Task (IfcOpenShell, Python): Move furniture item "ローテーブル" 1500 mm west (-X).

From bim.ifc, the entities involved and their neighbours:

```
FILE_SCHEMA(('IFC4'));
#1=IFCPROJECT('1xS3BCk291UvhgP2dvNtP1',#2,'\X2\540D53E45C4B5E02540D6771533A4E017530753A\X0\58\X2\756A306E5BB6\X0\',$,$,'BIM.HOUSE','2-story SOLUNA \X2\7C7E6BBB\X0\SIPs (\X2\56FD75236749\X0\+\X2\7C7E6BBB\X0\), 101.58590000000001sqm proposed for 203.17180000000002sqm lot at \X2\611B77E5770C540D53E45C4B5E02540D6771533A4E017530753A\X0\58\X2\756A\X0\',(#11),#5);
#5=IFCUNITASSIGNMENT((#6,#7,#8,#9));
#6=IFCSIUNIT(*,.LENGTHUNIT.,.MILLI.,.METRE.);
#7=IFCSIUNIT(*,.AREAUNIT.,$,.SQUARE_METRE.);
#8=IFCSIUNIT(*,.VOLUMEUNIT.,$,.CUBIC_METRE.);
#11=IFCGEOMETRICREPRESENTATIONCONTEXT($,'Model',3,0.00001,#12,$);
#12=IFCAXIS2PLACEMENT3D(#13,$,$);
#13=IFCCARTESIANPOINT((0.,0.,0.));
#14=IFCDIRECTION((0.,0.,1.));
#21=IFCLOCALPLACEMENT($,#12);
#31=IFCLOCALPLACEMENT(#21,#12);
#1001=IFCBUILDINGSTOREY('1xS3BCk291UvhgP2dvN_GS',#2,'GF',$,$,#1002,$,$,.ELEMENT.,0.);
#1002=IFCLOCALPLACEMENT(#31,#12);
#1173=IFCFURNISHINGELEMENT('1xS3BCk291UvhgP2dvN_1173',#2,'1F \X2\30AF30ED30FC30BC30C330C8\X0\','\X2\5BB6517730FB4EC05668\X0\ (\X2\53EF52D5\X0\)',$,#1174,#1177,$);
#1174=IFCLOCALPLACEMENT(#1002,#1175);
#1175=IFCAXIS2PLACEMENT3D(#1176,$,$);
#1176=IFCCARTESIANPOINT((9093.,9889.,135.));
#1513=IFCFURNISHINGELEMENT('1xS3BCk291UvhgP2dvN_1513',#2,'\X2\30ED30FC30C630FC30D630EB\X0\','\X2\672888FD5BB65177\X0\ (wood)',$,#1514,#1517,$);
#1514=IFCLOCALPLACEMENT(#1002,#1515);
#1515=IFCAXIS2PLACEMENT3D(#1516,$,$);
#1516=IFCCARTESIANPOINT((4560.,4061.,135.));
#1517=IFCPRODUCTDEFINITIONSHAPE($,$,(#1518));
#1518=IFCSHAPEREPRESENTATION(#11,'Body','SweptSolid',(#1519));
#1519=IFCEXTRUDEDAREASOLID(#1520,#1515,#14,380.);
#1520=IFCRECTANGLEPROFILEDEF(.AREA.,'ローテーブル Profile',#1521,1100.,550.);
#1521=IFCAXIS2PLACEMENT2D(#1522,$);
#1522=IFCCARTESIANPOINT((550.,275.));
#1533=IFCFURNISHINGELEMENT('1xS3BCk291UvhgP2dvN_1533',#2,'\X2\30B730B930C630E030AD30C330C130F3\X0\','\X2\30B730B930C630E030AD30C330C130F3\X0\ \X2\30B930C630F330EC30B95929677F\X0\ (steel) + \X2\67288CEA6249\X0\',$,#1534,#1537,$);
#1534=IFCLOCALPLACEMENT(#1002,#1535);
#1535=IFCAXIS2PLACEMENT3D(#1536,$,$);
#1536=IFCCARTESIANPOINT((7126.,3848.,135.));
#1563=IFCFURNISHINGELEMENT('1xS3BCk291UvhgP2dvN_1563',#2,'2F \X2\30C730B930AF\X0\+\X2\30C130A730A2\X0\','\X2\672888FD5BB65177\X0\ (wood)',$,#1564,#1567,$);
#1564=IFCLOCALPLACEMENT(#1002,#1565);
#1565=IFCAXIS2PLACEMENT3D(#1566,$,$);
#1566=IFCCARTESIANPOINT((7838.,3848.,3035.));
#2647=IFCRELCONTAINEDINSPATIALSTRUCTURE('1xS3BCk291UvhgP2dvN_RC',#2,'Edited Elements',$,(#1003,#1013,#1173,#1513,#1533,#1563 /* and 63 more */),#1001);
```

```python
import ifcopenshell
import ifcopenshell.api.geometry
import ifcopenshell.util.placement
import ifcopenshell.util.unit

model = ifcopenshell.open("bim.ifc")
unit_scale = ifcopenshell.util.unit.calculate_unit_scale(model)

item = model.by_guid("1xS3BCk291UvhgP2dvN_1513")
matrix = ifcopenshell.util.placement.get_local_placement(item.ObjectPlacement)
matrix[0, 3] -= 1.5 / unit_scale
ifcopenshell.api.geometry.edit_object_placement(model, product=item, matrix=matrix, is_si=False)

print(ifcopenshell.util.placement.get_local_placement(item.ObjectPlacement).round(3) + 0.0)

model.write("bim_rev.ifc")
```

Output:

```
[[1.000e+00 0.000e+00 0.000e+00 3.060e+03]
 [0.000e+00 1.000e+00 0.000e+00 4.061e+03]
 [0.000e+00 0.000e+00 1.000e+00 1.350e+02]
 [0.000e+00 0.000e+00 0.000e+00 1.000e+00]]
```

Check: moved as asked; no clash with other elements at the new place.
